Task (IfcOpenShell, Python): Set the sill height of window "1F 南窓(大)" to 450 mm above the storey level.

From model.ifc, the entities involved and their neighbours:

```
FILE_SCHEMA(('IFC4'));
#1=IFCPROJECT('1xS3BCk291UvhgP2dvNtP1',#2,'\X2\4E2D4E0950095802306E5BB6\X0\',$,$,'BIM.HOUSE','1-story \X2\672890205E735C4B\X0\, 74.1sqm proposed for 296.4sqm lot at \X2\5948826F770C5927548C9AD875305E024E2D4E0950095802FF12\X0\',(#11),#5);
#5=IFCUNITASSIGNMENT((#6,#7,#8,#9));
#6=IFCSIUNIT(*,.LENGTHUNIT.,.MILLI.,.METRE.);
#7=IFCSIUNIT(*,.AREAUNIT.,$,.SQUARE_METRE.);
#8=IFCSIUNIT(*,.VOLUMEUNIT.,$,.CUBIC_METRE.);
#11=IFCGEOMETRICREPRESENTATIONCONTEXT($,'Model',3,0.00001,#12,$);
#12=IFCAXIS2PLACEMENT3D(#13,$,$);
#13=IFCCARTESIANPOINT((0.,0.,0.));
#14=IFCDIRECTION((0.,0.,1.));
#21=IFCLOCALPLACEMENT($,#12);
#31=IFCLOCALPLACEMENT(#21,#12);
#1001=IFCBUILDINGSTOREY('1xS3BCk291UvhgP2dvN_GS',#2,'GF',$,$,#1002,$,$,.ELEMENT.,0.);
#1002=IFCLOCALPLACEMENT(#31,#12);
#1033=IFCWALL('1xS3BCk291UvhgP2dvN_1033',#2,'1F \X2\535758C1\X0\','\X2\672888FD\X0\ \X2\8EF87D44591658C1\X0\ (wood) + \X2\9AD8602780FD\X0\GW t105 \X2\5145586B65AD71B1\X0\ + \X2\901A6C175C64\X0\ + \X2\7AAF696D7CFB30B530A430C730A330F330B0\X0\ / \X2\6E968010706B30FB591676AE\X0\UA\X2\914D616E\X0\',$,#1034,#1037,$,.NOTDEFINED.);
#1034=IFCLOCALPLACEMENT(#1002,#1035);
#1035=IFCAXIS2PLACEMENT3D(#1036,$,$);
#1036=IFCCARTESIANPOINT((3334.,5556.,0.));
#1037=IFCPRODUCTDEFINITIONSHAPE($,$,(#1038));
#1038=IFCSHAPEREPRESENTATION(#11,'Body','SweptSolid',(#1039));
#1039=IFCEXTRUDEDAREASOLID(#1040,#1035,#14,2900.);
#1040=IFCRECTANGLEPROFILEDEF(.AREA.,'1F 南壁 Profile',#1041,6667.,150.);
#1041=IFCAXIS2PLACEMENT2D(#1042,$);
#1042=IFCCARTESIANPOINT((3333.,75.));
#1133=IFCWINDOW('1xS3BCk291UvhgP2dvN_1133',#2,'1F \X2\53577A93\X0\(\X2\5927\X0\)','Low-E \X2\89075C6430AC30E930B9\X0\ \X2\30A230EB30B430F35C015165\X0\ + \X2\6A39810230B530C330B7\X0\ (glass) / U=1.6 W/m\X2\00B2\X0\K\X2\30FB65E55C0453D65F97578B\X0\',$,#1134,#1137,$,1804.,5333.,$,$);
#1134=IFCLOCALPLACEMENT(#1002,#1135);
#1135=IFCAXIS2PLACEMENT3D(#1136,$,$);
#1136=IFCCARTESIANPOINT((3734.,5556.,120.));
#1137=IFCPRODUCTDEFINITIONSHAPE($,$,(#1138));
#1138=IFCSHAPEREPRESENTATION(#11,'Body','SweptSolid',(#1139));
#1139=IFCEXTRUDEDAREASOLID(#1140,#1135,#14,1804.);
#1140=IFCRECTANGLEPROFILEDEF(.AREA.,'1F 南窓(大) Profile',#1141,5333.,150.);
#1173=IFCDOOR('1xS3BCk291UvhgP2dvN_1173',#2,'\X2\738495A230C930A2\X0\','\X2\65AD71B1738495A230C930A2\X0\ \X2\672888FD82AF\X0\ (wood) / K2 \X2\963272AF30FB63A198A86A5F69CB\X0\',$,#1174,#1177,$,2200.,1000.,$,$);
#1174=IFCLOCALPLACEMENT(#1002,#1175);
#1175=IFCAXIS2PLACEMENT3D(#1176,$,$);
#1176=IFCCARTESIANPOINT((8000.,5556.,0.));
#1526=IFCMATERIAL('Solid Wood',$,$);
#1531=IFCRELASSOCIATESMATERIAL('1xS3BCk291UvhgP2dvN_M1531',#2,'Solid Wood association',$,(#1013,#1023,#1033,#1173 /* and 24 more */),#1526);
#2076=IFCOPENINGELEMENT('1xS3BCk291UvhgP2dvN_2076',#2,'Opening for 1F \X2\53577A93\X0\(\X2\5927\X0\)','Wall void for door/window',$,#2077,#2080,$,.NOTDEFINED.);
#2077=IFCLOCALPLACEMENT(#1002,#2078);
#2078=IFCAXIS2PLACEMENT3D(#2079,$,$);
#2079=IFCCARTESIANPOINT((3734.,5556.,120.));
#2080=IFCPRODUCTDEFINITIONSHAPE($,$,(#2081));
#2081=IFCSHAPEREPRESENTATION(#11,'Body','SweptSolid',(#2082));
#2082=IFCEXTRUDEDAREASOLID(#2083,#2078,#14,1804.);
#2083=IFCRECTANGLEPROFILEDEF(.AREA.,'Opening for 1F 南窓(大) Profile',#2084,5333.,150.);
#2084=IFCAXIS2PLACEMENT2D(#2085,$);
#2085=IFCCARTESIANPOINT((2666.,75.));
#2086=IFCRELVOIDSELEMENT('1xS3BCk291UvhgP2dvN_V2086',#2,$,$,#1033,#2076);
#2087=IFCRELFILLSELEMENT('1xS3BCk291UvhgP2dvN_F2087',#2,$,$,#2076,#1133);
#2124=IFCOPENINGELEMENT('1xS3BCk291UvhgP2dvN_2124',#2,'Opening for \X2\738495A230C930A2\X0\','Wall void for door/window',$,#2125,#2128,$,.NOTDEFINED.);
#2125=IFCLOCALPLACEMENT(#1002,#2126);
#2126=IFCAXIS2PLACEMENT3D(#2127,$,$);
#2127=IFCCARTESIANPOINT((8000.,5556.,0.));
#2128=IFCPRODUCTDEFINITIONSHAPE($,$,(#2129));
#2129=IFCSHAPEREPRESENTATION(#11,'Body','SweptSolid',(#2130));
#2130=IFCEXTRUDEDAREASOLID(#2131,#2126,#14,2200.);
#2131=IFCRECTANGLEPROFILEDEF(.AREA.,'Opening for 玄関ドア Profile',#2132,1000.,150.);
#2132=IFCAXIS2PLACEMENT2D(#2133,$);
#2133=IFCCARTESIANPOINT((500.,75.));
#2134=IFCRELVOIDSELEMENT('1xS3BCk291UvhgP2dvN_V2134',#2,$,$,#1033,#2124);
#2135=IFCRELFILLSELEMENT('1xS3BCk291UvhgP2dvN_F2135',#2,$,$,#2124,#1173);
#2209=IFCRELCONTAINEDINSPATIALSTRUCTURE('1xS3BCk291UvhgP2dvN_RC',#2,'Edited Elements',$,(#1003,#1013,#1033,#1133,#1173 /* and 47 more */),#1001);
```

```python
import numpy as np
import ifcopenshell
import ifcopenshell.api.geometry
import ifcopenshell.geom
import ifcopenshell.util.element
import ifcopenshell.util.placement
import ifcopenshell.util.shape
import ifcopenshell.util.unit

model = ifcopenshell.open("model.ifc")
unit_scale = ifcopenshell.util.unit.calculate_unit_scale(model)

window = model.by_id(1133)
opening = window.FillsVoids[0].RelatingOpeningElement
storey = ifcopenshell.util.element.get_container(window, ifc_class="IfcBuildingStorey")
level = ifcopenshell.util.placement.get_local_placement(storey.ObjectPlacement)[2, 3]

# The opening's origin need not be at the sill, so measure its lowest point.
shape = ifcopenshell.geom.create_shape(ifcopenshell.geom.settings(), opening)
bottom = ifcopenshell.util.shape.get_shape_bottom_elevation(shape, shape.geometry) / unit_scale
dz = level + 0.45 / unit_scale - bottom

shift = np.array([0.0, 0.0, dz])
# The window is not placed relative to its opening, so move both.
for product in (opening, window):
    matrix = ifcopenshell.util.placement.get_local_placement(product.ObjectPlacement)
    matrix[:3, 3] += shift
    ifcopenshell.api.geometry.edit_object_placement(model, product=product, matrix=matrix, is_si=False)

print(f"moved by {dz * unit_scale:+.3f} m")

model.write("model_v2.ifc")
```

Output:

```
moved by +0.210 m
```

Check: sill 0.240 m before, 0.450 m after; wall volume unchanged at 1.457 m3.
